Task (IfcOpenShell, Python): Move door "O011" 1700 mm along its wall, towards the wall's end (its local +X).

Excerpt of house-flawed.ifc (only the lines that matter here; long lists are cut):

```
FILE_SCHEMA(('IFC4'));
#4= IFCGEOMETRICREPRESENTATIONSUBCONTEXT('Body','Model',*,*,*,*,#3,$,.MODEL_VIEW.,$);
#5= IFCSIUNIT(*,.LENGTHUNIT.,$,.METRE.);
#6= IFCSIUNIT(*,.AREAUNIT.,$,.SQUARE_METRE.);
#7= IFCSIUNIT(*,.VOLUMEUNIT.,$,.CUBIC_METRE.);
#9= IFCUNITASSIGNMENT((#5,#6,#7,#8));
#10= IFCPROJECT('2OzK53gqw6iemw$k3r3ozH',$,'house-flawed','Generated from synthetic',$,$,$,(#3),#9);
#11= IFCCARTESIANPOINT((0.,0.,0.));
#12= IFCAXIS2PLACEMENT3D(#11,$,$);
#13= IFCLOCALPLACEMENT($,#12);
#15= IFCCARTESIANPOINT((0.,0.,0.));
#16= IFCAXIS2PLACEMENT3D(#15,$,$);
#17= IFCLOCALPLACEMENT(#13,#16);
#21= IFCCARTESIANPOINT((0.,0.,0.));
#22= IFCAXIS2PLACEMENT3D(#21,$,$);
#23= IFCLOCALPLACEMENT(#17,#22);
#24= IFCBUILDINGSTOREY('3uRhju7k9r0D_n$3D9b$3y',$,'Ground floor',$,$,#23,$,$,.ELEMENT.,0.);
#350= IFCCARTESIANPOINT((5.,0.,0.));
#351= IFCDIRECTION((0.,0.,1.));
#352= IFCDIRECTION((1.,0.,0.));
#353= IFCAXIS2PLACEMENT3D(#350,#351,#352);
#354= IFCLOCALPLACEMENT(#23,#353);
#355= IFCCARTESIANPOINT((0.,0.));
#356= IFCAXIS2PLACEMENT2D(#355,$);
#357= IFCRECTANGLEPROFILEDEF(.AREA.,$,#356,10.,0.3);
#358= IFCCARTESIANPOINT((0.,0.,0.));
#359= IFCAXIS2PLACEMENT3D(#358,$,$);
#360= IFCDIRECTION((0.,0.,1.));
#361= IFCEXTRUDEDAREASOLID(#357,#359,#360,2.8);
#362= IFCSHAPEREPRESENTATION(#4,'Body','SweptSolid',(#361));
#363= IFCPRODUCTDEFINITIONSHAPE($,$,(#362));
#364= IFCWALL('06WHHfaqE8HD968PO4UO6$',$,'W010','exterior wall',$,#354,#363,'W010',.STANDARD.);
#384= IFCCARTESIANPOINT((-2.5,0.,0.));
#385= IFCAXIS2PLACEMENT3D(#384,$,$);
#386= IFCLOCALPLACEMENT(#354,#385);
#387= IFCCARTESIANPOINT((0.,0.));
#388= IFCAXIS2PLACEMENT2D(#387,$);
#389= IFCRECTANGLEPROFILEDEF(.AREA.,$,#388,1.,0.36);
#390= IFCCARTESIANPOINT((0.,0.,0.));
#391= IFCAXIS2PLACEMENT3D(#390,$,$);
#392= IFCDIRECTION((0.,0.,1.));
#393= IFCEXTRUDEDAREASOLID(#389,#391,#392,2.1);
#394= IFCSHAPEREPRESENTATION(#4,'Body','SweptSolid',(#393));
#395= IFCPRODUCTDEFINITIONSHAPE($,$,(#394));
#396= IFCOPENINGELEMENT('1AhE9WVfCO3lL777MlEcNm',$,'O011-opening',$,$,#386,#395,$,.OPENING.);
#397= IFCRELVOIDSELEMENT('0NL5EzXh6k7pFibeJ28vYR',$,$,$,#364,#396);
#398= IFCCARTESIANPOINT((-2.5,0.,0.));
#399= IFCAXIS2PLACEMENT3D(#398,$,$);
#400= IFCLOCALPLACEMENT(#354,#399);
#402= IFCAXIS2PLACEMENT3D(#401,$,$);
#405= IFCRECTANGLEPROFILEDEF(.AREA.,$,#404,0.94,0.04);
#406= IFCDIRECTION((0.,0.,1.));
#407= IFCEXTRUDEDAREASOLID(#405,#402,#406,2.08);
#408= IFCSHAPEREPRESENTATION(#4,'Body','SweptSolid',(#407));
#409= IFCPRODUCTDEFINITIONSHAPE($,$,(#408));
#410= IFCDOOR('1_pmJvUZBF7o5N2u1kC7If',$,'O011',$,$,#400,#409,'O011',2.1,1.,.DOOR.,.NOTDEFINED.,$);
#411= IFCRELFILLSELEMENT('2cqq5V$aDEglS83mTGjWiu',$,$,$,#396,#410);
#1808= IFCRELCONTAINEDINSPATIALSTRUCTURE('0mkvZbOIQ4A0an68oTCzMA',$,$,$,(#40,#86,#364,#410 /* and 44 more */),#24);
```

```python
import ifcopenshell
import ifcopenshell.api.geometry
import ifcopenshell.util.placement

model = ifcopenshell.open("house-flawed.ifc")

door = model.by_id(410)
opening = door.FillsVoids[0].RelatingOpeningElement
wall = opening.VoidsElements[0].RelatingBuildingElement

wall_matrix = ifcopenshell.util.placement.get_local_placement(wall.ObjectPlacement)
shift = wall_matrix[:3, 0] * 1.7
before = ifcopenshell.util.placement.get_local_placement(door.ObjectPlacement)[:3, 3].copy()

# The door is not placed relative to its opening, so move both.
for product in (opening, door):
    matrix = ifcopenshell.util.placement.get_local_placement(product.ObjectPlacement)
    matrix[:3, 3] += shift
    ifcopenshell.api.geometry.edit_object_placement(model, product=product, matrix=matrix, is_si=False)

after = ifcopenshell.util.placement.get_local_placement(door.ObjectPlacement)[:3, 3]
print("door moved by", (after - before).round(3) + 0.0)

model.write("house-flawed_edited.ifc")
```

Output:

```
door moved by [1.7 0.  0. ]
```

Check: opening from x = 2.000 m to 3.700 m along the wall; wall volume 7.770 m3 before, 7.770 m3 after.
